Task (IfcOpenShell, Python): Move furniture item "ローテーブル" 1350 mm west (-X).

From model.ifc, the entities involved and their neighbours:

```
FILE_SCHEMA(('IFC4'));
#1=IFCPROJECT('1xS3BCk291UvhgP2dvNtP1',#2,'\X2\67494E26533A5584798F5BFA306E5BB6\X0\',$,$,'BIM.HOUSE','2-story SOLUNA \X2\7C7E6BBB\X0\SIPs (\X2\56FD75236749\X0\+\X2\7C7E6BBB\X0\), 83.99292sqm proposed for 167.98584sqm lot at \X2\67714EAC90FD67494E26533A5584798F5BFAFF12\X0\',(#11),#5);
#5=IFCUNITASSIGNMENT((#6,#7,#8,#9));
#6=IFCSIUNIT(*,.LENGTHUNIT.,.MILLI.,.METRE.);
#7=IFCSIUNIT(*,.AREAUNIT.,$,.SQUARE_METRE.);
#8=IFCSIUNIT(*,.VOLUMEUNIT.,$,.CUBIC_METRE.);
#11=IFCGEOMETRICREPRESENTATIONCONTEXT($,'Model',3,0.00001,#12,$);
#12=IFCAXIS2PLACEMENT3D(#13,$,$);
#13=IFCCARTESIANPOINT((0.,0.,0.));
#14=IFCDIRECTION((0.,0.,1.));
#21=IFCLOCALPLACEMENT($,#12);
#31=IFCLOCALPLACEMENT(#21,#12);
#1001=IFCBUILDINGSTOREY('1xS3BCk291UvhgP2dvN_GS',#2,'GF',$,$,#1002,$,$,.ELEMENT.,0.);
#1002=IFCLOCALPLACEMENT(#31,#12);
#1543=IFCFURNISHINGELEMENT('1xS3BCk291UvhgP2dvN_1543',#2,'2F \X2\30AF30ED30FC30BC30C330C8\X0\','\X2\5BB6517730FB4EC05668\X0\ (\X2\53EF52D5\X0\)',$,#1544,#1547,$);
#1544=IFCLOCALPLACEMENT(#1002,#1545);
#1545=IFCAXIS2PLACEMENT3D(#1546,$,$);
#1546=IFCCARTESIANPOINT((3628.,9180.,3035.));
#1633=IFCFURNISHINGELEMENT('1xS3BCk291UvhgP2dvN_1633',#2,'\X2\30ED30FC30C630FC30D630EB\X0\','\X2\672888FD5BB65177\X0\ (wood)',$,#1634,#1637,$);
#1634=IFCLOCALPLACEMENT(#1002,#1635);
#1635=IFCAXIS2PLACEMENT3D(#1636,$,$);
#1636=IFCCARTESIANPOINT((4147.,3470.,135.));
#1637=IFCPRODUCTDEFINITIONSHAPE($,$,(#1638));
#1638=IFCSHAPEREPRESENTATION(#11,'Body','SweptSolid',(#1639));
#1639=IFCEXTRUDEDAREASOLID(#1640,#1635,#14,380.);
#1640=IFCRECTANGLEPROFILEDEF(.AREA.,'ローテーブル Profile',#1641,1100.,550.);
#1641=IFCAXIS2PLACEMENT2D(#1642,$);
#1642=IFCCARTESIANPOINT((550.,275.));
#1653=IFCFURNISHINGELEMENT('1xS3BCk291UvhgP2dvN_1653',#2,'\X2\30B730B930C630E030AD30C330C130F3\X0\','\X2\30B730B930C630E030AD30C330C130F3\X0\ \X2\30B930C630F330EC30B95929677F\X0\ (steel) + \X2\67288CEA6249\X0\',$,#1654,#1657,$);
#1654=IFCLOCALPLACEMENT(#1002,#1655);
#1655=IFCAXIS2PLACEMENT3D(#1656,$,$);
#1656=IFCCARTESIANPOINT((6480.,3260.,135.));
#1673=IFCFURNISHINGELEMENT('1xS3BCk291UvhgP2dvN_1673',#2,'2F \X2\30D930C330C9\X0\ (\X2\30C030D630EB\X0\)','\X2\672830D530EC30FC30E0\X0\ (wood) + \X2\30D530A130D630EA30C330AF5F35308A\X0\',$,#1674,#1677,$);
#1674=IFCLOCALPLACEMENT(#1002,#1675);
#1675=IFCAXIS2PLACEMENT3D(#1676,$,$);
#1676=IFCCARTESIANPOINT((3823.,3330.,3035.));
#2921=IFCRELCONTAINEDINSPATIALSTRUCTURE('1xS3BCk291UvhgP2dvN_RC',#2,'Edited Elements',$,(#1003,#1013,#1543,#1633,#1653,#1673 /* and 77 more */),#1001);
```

```python
import ifcopenshell
import ifcopenshell.api.geometry
import ifcopenshell.util.placement
import ifcopenshell.util.unit

model = ifcopenshell.open("model.ifc")
unit_scale = ifcopenshell.util.unit.calculate_unit_scale(model)

item = model.by_guid("1xS3BCk291UvhgP2dvN_1633")
matrix = ifcopenshell.util.placement.get_local_placement(item.ObjectPlacement)
matrix[0, 3] -= 1.35 / unit_scale
ifcopenshell.api.geometry.edit_object_placement(model, product=item, matrix=matrix, is_si=False)

print(ifcopenshell.util.placement.get_local_placement(item.ObjectPlacement).round(3) + 0.0)

model.write("model_rev.ifc")
```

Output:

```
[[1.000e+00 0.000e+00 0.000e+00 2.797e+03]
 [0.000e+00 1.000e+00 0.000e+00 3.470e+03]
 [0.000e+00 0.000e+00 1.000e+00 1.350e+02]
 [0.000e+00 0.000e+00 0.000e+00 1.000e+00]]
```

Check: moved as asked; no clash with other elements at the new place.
